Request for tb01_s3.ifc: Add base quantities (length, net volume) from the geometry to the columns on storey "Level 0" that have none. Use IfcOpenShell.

First a look at what the model holds.

```python
import ifcopenshell
import ifcopenshell.util.element
import ifcopenshell.util.unit

model = ifcopenshell.open("tb01_s3.ifc")
print(model.schema)
for unit_type in ("LENGTHUNIT", "AREAUNIT", "VOLUMEUNIT"):
    print(unit_type, ifcopenshell.util.unit.calculate_unit_scale(model, unit_type))
storey = next(s for s in model.by_type("IfcBuildingStorey") if s.Name == "Level 0")
columns = [e for e in ifcopenshell.util.element.get_decomposition(storey) if e.is_a("IfcColumn")]
for e in sorted(columns, key=lambda e: e.id()):
    print(e.id(), e.is_a(), e.Name, list(ifcopenshell.util.element.get_psets(e, qtos_only=True)), sep=" | ")
```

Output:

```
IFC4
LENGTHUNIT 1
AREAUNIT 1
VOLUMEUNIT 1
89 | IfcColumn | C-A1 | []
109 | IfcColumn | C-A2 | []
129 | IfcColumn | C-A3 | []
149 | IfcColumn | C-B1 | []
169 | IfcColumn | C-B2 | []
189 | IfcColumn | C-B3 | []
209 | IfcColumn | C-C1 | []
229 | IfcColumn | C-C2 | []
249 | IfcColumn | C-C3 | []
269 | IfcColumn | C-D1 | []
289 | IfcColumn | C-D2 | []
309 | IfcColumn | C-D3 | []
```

```python
import ifcopenshell
import ifcopenshell.api.pset
import ifcopenshell.geom
import ifcopenshell.util.element
import ifcopenshell.util.shape
import ifcopenshell.util.unit

model = ifcopenshell.open("tb01_s3.ifc")
unit_scale = ifcopenshell.util.unit.calculate_unit_scale(model)
volume_scale = ifcopenshell.util.unit.calculate_unit_scale(model, "VOLUMEUNIT")
settings = ifcopenshell.geom.settings()

storey = next(s for s in model.by_type("IfcBuildingStorey") if s.Name == "Level 0")
columns = [e for e in ifcopenshell.util.element.get_decomposition(storey) if e.is_a("IfcColumn")]

for e in sorted(columns, key=lambda e: e.id()):
    if ifcopenshell.util.element.get_psets(e, qtos_only=True, should_inherit=False):
        continue
    # Geometry comes back in metres, in the element's own axes.
    shape = ifcopenshell.geom.create_shape(settings, e)
    values = {
        "Length": ifcopenshell.util.shape.get_z(shape.geometry) / unit_scale,
        "NetVolume": ifcopenshell.util.shape.get_volume(shape.geometry) / volume_scale,
    }
    qto = ifcopenshell.api.pset.add_qto(model, product=e, name="Qto_ColumnBaseQuantities")
    ifcopenshell.api.pset.edit_qto(model, qto=qto, properties=values)
    print(e.id(), {k: round(v, 3) for k, v in values.items()})

model.write("tb01_s3_updated.ifc")
```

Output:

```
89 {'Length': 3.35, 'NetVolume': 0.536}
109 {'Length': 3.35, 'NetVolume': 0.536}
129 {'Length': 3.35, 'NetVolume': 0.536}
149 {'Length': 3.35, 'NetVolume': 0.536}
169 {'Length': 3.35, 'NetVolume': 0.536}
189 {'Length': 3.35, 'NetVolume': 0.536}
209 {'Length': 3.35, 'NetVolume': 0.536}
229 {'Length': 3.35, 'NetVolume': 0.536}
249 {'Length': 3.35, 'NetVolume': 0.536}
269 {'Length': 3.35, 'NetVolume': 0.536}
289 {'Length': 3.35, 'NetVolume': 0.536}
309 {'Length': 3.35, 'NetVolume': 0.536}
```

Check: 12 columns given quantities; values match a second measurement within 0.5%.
